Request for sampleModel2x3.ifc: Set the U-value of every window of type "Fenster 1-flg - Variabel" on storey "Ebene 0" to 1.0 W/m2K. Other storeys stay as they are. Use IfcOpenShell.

First a look at what the model holds.

```python
import ifcopenshell
import ifcopenshell.util.element

model = ifcopenshell.open("sampleModel2x3.ifc")
print(model.schema)
storey = next(s for s in model.by_type("IfcBuildingStorey") if s.Name == "Ebene 0")
windows = [e for e in ifcopenshell.util.element.get_decomposition(storey) if e.is_a("IfcWindow")]
seen = {}
for e in windows:
    element_type = ifcopenshell.util.element.get_type(e)
    key = (element_type.Name if element_type != e and element_type else None, ifcopenshell.util.element.get_pset(e, "Pset_WindowCommon", "ThermalTransmittance"))
    seen[key] = seen.get(key, 0) + 1
for (name, value), count in sorted(seen.items(), key=str):
    print(count, "x", name, "|", value)
```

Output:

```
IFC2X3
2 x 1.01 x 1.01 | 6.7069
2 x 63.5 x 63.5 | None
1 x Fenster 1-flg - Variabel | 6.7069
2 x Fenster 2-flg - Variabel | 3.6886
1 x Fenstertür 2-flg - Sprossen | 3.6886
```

```python
import ifcopenshell
import ifcopenshell.api.pset
import ifcopenshell.util.element

model = ifcopenshell.open("sampleModel2x3.ifc")

storey = next(s for s in model.by_type("IfcBuildingStorey") if s.Name == "Ebene 0")
windows = [e for e in ifcopenshell.util.element.get_decomposition(storey) if e.is_a("IfcWindow")]

count = 0
for e in windows:
    element_type = ifcopenshell.util.element.get_type(e)
    if element_type in (None, e) or element_type.Name != "Fenster 1-flg - Variabel":
        continue
    # add_pset returns the element's existing set when there is one.
    pset = ifcopenshell.api.pset.add_pset(model, product=e, name="Pset_WindowCommon")
    ifcopenshell.api.pset.edit_pset(model, pset=pset, properties={"ThermalTransmittance": 1.0})
    count += 1

print(count, "windows updated")

model.write("sampleModel2x3_edited.ifc")
```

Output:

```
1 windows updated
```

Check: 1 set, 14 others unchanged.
